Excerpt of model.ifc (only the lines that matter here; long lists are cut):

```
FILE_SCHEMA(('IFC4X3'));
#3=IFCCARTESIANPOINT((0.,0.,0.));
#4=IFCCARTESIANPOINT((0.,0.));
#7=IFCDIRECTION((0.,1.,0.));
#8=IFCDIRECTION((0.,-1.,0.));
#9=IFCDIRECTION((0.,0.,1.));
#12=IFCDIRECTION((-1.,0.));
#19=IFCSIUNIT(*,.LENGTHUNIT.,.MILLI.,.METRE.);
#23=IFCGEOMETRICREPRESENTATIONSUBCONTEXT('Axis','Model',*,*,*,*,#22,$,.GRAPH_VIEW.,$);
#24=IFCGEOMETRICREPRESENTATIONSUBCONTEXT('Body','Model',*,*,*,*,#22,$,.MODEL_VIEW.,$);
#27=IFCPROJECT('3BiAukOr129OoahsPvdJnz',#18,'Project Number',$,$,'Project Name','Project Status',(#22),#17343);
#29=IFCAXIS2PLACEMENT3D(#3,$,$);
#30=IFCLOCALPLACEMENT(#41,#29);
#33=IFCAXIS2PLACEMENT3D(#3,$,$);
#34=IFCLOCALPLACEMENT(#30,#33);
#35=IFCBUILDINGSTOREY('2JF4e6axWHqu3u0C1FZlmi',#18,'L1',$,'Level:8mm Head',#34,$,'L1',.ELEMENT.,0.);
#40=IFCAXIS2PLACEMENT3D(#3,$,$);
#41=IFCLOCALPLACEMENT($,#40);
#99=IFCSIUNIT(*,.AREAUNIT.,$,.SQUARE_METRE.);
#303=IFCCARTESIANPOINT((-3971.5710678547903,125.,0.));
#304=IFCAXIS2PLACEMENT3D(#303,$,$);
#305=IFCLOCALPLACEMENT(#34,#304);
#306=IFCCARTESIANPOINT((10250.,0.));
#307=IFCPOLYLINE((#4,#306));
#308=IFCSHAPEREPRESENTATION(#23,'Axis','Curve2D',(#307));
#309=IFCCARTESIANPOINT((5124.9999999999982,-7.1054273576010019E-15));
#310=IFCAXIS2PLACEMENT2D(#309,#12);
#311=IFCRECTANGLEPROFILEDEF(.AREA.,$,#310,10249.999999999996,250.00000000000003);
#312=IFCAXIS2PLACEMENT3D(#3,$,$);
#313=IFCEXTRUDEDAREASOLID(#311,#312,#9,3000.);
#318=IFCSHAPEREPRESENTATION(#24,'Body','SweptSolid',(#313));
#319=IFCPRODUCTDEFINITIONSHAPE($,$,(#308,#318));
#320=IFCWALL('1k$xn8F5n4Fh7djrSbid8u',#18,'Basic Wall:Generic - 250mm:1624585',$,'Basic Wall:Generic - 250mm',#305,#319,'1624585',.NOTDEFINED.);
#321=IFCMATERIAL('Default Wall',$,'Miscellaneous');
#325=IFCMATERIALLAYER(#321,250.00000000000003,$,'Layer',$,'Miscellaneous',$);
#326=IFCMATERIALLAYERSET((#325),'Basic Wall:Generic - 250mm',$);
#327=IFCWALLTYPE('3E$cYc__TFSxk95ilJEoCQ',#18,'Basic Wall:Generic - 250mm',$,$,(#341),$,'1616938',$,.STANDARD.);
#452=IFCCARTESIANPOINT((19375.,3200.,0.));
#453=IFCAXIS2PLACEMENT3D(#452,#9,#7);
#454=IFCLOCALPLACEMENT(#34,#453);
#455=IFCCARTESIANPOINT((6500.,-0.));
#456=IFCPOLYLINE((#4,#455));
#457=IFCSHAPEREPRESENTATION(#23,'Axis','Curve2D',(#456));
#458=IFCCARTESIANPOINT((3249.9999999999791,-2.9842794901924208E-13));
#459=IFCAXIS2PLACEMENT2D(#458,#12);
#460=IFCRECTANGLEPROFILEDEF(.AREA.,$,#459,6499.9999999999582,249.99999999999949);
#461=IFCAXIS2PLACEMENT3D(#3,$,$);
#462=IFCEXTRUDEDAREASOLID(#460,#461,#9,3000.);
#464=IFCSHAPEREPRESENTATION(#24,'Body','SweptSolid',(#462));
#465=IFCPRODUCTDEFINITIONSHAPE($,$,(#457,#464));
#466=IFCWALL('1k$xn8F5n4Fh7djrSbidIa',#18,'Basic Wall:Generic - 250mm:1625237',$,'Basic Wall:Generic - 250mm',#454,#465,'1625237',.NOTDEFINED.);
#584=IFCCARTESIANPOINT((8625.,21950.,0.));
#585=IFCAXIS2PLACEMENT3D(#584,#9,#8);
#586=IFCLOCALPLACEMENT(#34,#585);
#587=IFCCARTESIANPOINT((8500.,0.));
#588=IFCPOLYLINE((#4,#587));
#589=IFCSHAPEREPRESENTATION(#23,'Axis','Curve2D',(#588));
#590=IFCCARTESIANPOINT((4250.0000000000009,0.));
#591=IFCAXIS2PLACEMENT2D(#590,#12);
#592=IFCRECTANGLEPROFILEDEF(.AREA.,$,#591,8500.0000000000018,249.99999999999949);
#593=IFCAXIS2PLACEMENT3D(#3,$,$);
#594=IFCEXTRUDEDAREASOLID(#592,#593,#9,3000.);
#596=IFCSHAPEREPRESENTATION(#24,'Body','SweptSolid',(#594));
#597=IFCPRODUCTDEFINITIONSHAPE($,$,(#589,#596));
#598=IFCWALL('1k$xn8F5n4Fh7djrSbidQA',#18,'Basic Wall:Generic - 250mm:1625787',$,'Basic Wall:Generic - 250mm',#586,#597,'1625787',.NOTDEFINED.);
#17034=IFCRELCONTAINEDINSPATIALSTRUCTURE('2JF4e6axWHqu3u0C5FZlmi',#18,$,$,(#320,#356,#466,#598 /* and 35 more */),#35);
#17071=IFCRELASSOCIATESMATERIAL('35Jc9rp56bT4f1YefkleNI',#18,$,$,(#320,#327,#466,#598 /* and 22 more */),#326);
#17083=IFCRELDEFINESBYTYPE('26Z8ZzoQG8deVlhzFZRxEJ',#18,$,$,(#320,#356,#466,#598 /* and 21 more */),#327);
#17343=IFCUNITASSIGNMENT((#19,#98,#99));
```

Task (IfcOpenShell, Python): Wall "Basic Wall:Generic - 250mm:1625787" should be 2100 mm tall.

```python
import ifcopenshell
import ifcopenshell.geom
import ifcopenshell.util.representation
import ifcopenshell.util.shape

model = ifcopenshell.open("model.ifc")
settings = ifcopenshell.geom.settings()


def volume(element):
    """Net volume in cubic metres, openings subtracted."""
    shape = ifcopenshell.geom.create_shape(settings, element)
    return ifcopenshell.util.shape.get_volume(shape.geometry)


wall = model.by_guid("1k$xn8F5n4Fh7djrSbidQA")
before = volume(wall)

body = ifcopenshell.util.representation.get_representation(wall, "Model", "Body")
solid = body.Items[0]
old_height = solid.Depth
solid.Depth = 2100.0
after = volume(wall)

print(f"height {old_height:g} -> {solid.Depth:g}, volume {before:.3f} -> {after:.3f} m3")

model.write("model_updated.ifc")
```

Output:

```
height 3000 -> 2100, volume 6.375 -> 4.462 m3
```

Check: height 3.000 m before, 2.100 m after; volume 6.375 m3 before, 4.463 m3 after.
